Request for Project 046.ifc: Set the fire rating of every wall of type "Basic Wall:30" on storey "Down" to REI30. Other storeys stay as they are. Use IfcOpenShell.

First a look at what the model holds.

```python
import ifcopenshell
import ifcopenshell.util.element

model = ifcopenshell.open("Project 046.ifc")
print(model.schema)
storey = next(s for s in model.by_type("IfcBuildingStorey") if s.Name == "Down")
walls = [e for e in ifcopenshell.util.element.get_decomposition(storey) if e.is_a("IfcWall")]
seen = {}
for e in walls:
    element_type = ifcopenshell.util.element.get_type(e)
    key = (element_type.Name if element_type != e and element_type else None, ifcopenshell.util.element.get_pset(e, "Pset_WallCommon", "FireRating"))
    seen[key] = seen.get(key, 0) + 1
for (name, value), count in sorted(seen.items(), key=str):
    print(count, "x", name, "|", value)
```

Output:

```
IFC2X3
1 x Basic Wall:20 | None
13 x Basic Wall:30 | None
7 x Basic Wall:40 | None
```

```python
import ifcopenshell
import ifcopenshell.api.pset
import ifcopenshell.util.element

model = ifcopenshell.open("Project 046.ifc")

storey = next(s for s in model.by_type("IfcBuildingStorey") if s.Name == "Down")
walls = [e for e in ifcopenshell.util.element.get_decomposition(storey) if e.is_a("IfcWall")]

count = 0
for e in walls:
    element_type = ifcopenshell.util.element.get_type(e)
    if element_type in (None, e) or element_type.Name != "Basic Wall:30":
        continue
    # add_pset returns the element's existing set when there is one.
    pset = ifcopenshell.api.pset.add_pset(model, product=e, name="Pset_WallCommon")
    ifcopenshell.api.pset.edit_pset(model, pset=pset, properties={"FireRating": "REI30"})
    count += 1

print(count, "walls updated")

model.write("Project 046_updated.ifc")
```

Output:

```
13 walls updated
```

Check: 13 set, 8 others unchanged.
